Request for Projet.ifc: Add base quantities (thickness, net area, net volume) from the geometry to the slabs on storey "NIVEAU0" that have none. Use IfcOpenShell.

First a look at what the model holds.

```python
import ifcopenshell
import ifcopenshell.util.element
import ifcopenshell.util.unit

model = ifcopenshell.open("Projet.ifc")
print(model.schema)
for unit_type in ("LENGTHUNIT", "AREAUNIT", "VOLUMEUNIT"):
    print(unit_type, ifcopenshell.util.unit.calculate_unit_scale(model, unit_type))
storey = next(s for s in model.by_type("IfcBuildingStorey") if s.Name == "NIVEAU0")
slabs = [e for e in ifcopenshell.util.element.get_decomposition(storey) if e.is_a("IfcSlab")]
for e in sorted(slabs, key=lambda e: e.id()):
    print(e.id(), e.is_a(), e.Name, list(ifcopenshell.util.element.get_psets(e, qtos_only=True)), sep=" | ")
```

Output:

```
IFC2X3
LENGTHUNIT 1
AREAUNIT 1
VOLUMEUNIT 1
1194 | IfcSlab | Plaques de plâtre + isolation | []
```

```python
import ifcopenshell
import ifcopenshell.api.pset
import ifcopenshell.geom
import ifcopenshell.util.element
import ifcopenshell.util.shape
import ifcopenshell.util.unit

model = ifcopenshell.open("Projet.ifc")
unit_scale = ifcopenshell.util.unit.calculate_unit_scale(model)
area_scale = ifcopenshell.util.unit.calculate_unit_scale(model, "AREAUNIT")
volume_scale = ifcopenshell.util.unit.calculate_unit_scale(model, "VOLUMEUNIT")
settings = ifcopenshell.geom.settings()

storey = next(s for s in model.by_type("IfcBuildingStorey") if s.Name == "NIVEAU0")
slabs = [e for e in ifcopenshell.util.element.get_decomposition(storey) if e.is_a("IfcSlab")]

for e in sorted(slabs, key=lambda e: e.id()):
    if ifcopenshell.util.element.get_psets(e, qtos_only=True, should_inherit=False):
        continue
    # Geometry comes back in metres, in the element's own axes.
    shape = ifcopenshell.geom.create_shape(settings, e)
    values = {
        "Width": ifcopenshell.util.shape.get_z(shape.geometry) / unit_scale,
        "NetArea": ifcopenshell.util.shape.get_footprint_area(shape.geometry) / area_scale,
        "NetVolume": ifcopenshell.util.shape.get_volume(shape.geometry) / volume_scale,
    }
    qto = ifcopenshell.api.pset.add_qto(model, product=e, name="BaseQuantities")
    ifcopenshell.api.pset.edit_qto(model, qto=qto, properties=values)
    print(e.id(), {k: round(v, 3) for k, v in values.items()})

model.write("Projet_rev.ifc")
```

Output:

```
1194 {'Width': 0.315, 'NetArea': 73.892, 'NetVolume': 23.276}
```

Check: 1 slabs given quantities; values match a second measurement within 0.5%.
